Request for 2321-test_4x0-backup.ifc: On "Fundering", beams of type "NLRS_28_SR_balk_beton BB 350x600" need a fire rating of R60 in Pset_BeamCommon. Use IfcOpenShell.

First a look at what the model holds.

```python
import ifcopenshell
import ifcopenshell.util.element

model = ifcopenshell.open("2321-test_4x0-backup.ifc")
print(model.schema)
storey = next(s for s in model.by_type("IfcBuildingStorey") if s.Name == "Fundering")
beams = [e for e in ifcopenshell.util.element.get_decomposition(storey) if e.is_a("IfcBeam")]
seen = {}
for e in beams:
    element_type = ifcopenshell.util.element.get_type(e)
    key = (element_type.Name if element_type != e and element_type else None, ifcopenshell.util.element.get_pset(e, "Pset_BeamCommon", "FireRating"))
    seen[key] = seen.get(key, 0) + 1
for (name, value), count in sorted(seen.items(), key=str):
    print(count, "x", name, "|", value)
```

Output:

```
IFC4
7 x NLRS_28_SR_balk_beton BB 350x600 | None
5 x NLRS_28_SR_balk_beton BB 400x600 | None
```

```python
import ifcopenshell
import ifcopenshell.api.pset
import ifcopenshell.util.element

model = ifcopenshell.open("2321-test_4x0-backup.ifc")

storey = next(s for s in model.by_type("IfcBuildingStorey") if s.Name == "Fundering")
beams = [e for e in ifcopenshell.util.element.get_decomposition(storey) if e.is_a("IfcBeam")]

count = 0
for e in beams:
    element_type = ifcopenshell.util.element.get_type(e)
    if element_type in (None, e) or element_type.Name != "NLRS_28_SR_balk_beton BB 350x600":
        continue
    # add_pset returns the element's existing set when there is one.
    pset = ifcopenshell.api.pset.add_pset(model, product=e, name="Pset_BeamCommon")
    ifcopenshell.api.pset.edit_pset(model, pset=pset, properties={"FireRating": "R60"})
    count += 1

print(count, "beams updated")

model.write("2321-test_4x0-backup_rev.ifc")
```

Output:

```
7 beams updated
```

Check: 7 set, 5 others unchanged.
